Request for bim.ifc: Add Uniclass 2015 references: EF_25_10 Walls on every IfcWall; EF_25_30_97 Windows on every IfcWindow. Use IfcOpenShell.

First a look at what the model holds.

```python
import ifcopenshell

model = ifcopenshell.open("bim.ifc")
print(model.schema)
print("classifications:", [c.Name for c in model.by_type("IfcClassification")])
for ifc_class in ("IfcDoor", "IfcRoof", "IfcStair", "IfcWall", "IfcWindow"):
    print(ifc_class, len(model.by_type(ifc_class)))
```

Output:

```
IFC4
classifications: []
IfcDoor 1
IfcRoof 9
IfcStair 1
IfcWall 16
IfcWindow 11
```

```python
import ifcopenshell
import ifcopenshell.api.classification

model = ifcopenshell.open("bim.ifc")

system = ifcopenshell.api.classification.add_classification(model, classification="Uniclass 2015")

codes = {
    "IfcWall": ("EF_25_10", "Walls"),
    "IfcWindow": ("EF_25_30_97", "Windows"),
}
for ifc_class, (code, name) in codes.items():
    products = model.by_type(ifc_class)
    ifcopenshell.api.classification.add_reference(
        model, products=products, classification=system, identification=code, name=name
    )
    print(code, len(products))

model.write("bim_rev.ifc")
```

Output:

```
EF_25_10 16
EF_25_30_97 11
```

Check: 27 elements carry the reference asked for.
